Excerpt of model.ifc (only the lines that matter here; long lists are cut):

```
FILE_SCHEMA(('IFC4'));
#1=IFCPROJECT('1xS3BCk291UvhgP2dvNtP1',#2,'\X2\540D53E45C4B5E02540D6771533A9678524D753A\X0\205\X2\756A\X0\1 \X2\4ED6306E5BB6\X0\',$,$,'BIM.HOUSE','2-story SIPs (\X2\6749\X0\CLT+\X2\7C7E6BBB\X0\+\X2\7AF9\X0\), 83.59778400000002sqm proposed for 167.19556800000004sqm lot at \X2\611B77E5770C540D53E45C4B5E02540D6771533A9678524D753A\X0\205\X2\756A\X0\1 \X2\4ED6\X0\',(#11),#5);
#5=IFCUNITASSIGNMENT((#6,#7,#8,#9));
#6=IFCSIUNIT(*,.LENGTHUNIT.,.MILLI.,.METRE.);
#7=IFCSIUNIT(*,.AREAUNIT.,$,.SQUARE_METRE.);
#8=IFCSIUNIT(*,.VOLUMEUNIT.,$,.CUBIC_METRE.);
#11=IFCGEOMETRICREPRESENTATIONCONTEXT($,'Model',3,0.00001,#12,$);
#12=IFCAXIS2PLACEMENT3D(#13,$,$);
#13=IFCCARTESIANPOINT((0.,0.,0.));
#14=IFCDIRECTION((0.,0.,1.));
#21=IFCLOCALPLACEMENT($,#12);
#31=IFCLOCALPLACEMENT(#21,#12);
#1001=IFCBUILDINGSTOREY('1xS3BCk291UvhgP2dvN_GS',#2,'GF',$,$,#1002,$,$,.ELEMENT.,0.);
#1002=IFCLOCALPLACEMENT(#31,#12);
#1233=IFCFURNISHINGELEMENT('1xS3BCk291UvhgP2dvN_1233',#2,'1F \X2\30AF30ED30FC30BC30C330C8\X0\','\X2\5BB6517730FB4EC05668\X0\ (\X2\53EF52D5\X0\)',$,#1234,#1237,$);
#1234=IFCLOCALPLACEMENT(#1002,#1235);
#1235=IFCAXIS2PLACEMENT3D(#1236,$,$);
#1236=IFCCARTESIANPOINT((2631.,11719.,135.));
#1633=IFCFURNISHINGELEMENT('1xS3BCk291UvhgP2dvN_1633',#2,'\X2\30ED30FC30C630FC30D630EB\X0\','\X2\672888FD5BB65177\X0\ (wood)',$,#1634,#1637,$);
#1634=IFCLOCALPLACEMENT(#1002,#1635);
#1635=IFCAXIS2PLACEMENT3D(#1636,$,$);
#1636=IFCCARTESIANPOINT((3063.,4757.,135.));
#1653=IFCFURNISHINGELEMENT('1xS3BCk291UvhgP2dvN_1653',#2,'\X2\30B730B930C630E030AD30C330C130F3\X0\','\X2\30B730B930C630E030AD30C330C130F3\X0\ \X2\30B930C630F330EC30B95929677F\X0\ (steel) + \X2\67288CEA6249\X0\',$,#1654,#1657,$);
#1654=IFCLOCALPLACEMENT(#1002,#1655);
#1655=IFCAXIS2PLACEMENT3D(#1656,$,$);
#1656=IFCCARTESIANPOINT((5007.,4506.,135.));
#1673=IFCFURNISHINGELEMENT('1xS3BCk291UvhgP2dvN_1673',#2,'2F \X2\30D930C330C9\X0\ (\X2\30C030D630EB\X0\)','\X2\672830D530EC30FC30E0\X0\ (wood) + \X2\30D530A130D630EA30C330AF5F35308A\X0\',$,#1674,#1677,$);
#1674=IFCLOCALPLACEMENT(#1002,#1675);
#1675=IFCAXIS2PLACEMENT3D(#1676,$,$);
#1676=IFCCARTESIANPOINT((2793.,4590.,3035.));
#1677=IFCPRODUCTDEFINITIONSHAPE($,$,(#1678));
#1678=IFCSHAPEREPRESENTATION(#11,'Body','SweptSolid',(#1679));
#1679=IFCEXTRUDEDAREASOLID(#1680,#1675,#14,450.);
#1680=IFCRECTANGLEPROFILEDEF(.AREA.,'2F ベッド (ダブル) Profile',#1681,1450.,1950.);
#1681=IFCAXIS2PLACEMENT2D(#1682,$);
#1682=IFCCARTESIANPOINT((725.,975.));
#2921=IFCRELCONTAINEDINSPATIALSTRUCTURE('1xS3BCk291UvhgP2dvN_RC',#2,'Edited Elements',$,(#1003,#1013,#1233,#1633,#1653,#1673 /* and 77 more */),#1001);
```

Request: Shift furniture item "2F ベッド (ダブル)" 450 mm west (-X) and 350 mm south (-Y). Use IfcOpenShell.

```python
import ifcopenshell
import ifcopenshell.api.geometry
import ifcopenshell.util.placement
import ifcopenshell.util.unit

model = ifcopenshell.open("model.ifc")
unit_scale = ifcopenshell.util.unit.calculate_unit_scale(model)

item = model.by_guid("1xS3BCk291UvhgP2dvN_1673")
matrix = ifcopenshell.util.placement.get_local_placement(item.ObjectPlacement)
matrix[0, 3] -= 0.45 / unit_scale
matrix[1, 3] -= 0.35 / unit_scale
ifcopenshell.api.geometry.edit_object_placement(model, product=item, matrix=matrix, is_si=False)

print(ifcopenshell.util.placement.get_local_placement(item.ObjectPlacement).round(3) + 0.0)

model.write("model-out.ifc")
```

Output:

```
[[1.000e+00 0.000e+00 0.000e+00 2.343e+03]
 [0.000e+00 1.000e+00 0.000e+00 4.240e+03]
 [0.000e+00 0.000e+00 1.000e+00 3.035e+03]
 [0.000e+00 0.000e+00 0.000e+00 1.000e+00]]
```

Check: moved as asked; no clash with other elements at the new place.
